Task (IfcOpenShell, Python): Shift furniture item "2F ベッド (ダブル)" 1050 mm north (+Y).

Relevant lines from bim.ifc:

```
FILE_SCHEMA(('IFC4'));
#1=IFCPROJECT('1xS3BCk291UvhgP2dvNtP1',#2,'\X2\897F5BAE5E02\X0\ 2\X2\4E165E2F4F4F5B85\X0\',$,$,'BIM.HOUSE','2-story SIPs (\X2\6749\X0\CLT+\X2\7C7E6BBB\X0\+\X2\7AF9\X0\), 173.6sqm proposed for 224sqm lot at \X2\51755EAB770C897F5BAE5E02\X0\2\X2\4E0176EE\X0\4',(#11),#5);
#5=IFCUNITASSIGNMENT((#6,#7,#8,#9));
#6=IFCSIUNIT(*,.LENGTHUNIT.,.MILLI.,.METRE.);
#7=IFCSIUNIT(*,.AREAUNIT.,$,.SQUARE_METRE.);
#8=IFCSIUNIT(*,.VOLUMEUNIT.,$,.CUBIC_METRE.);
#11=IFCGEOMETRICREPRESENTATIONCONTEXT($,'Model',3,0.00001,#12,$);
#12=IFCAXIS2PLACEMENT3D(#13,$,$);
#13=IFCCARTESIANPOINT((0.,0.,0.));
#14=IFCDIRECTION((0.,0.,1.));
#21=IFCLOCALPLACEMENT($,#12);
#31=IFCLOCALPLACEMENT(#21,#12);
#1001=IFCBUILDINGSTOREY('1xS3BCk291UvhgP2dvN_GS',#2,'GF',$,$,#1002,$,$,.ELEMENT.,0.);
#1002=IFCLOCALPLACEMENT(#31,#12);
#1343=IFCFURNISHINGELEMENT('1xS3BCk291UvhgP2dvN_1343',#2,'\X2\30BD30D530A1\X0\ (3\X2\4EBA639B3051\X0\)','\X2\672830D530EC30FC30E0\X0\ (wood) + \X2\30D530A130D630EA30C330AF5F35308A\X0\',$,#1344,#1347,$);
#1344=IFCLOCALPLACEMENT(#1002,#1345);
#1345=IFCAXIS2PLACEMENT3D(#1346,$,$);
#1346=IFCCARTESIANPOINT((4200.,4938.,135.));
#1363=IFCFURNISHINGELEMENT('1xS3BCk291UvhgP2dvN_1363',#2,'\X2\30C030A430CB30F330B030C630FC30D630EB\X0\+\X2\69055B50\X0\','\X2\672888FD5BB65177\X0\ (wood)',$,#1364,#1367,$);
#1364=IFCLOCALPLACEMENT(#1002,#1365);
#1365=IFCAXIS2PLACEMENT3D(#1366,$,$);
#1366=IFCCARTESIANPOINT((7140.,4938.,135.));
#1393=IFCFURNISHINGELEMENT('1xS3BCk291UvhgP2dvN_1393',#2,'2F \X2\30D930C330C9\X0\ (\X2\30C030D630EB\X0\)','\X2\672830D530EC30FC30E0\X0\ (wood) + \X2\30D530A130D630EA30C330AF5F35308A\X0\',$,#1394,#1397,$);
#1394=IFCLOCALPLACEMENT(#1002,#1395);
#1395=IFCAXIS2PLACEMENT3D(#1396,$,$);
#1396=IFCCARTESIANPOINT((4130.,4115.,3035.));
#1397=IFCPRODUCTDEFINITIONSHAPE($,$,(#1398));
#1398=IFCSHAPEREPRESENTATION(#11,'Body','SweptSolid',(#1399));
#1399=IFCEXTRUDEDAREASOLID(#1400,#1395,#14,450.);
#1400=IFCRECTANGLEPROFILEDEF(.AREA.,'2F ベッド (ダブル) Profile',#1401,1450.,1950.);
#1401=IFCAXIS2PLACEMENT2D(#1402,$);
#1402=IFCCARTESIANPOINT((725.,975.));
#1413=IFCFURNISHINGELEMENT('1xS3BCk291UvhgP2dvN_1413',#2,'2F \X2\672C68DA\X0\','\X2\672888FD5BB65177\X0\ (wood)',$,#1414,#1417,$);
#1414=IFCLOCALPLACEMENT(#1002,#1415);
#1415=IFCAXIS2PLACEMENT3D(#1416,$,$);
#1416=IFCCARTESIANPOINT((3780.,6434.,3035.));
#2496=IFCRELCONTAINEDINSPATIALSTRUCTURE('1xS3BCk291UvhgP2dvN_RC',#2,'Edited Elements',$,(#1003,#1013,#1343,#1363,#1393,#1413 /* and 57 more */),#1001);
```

```python
import ifcopenshell
import ifcopenshell.api.geometry
import ifcopenshell.util.placement

model = ifcopenshell.open("bim.ifc")

item = model.by_guid("1xS3BCk291UvhgP2dvN_1393")
matrix = ifcopenshell.util.placement.get_local_placement(item.ObjectPlacement)
matrix[1, 3] += 1050.0
ifcopenshell.api.geometry.edit_object_placement(model, product=item, matrix=matrix, is_si=False)

print(ifcopenshell.util.placement.get_local_placement(item.ObjectPlacement).round(3) + 0.0)

model.write("bim_v2.ifc")
```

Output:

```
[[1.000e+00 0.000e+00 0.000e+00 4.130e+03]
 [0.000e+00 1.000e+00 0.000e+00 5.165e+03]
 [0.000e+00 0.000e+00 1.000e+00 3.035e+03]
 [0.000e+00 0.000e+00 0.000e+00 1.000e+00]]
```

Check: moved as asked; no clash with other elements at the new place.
